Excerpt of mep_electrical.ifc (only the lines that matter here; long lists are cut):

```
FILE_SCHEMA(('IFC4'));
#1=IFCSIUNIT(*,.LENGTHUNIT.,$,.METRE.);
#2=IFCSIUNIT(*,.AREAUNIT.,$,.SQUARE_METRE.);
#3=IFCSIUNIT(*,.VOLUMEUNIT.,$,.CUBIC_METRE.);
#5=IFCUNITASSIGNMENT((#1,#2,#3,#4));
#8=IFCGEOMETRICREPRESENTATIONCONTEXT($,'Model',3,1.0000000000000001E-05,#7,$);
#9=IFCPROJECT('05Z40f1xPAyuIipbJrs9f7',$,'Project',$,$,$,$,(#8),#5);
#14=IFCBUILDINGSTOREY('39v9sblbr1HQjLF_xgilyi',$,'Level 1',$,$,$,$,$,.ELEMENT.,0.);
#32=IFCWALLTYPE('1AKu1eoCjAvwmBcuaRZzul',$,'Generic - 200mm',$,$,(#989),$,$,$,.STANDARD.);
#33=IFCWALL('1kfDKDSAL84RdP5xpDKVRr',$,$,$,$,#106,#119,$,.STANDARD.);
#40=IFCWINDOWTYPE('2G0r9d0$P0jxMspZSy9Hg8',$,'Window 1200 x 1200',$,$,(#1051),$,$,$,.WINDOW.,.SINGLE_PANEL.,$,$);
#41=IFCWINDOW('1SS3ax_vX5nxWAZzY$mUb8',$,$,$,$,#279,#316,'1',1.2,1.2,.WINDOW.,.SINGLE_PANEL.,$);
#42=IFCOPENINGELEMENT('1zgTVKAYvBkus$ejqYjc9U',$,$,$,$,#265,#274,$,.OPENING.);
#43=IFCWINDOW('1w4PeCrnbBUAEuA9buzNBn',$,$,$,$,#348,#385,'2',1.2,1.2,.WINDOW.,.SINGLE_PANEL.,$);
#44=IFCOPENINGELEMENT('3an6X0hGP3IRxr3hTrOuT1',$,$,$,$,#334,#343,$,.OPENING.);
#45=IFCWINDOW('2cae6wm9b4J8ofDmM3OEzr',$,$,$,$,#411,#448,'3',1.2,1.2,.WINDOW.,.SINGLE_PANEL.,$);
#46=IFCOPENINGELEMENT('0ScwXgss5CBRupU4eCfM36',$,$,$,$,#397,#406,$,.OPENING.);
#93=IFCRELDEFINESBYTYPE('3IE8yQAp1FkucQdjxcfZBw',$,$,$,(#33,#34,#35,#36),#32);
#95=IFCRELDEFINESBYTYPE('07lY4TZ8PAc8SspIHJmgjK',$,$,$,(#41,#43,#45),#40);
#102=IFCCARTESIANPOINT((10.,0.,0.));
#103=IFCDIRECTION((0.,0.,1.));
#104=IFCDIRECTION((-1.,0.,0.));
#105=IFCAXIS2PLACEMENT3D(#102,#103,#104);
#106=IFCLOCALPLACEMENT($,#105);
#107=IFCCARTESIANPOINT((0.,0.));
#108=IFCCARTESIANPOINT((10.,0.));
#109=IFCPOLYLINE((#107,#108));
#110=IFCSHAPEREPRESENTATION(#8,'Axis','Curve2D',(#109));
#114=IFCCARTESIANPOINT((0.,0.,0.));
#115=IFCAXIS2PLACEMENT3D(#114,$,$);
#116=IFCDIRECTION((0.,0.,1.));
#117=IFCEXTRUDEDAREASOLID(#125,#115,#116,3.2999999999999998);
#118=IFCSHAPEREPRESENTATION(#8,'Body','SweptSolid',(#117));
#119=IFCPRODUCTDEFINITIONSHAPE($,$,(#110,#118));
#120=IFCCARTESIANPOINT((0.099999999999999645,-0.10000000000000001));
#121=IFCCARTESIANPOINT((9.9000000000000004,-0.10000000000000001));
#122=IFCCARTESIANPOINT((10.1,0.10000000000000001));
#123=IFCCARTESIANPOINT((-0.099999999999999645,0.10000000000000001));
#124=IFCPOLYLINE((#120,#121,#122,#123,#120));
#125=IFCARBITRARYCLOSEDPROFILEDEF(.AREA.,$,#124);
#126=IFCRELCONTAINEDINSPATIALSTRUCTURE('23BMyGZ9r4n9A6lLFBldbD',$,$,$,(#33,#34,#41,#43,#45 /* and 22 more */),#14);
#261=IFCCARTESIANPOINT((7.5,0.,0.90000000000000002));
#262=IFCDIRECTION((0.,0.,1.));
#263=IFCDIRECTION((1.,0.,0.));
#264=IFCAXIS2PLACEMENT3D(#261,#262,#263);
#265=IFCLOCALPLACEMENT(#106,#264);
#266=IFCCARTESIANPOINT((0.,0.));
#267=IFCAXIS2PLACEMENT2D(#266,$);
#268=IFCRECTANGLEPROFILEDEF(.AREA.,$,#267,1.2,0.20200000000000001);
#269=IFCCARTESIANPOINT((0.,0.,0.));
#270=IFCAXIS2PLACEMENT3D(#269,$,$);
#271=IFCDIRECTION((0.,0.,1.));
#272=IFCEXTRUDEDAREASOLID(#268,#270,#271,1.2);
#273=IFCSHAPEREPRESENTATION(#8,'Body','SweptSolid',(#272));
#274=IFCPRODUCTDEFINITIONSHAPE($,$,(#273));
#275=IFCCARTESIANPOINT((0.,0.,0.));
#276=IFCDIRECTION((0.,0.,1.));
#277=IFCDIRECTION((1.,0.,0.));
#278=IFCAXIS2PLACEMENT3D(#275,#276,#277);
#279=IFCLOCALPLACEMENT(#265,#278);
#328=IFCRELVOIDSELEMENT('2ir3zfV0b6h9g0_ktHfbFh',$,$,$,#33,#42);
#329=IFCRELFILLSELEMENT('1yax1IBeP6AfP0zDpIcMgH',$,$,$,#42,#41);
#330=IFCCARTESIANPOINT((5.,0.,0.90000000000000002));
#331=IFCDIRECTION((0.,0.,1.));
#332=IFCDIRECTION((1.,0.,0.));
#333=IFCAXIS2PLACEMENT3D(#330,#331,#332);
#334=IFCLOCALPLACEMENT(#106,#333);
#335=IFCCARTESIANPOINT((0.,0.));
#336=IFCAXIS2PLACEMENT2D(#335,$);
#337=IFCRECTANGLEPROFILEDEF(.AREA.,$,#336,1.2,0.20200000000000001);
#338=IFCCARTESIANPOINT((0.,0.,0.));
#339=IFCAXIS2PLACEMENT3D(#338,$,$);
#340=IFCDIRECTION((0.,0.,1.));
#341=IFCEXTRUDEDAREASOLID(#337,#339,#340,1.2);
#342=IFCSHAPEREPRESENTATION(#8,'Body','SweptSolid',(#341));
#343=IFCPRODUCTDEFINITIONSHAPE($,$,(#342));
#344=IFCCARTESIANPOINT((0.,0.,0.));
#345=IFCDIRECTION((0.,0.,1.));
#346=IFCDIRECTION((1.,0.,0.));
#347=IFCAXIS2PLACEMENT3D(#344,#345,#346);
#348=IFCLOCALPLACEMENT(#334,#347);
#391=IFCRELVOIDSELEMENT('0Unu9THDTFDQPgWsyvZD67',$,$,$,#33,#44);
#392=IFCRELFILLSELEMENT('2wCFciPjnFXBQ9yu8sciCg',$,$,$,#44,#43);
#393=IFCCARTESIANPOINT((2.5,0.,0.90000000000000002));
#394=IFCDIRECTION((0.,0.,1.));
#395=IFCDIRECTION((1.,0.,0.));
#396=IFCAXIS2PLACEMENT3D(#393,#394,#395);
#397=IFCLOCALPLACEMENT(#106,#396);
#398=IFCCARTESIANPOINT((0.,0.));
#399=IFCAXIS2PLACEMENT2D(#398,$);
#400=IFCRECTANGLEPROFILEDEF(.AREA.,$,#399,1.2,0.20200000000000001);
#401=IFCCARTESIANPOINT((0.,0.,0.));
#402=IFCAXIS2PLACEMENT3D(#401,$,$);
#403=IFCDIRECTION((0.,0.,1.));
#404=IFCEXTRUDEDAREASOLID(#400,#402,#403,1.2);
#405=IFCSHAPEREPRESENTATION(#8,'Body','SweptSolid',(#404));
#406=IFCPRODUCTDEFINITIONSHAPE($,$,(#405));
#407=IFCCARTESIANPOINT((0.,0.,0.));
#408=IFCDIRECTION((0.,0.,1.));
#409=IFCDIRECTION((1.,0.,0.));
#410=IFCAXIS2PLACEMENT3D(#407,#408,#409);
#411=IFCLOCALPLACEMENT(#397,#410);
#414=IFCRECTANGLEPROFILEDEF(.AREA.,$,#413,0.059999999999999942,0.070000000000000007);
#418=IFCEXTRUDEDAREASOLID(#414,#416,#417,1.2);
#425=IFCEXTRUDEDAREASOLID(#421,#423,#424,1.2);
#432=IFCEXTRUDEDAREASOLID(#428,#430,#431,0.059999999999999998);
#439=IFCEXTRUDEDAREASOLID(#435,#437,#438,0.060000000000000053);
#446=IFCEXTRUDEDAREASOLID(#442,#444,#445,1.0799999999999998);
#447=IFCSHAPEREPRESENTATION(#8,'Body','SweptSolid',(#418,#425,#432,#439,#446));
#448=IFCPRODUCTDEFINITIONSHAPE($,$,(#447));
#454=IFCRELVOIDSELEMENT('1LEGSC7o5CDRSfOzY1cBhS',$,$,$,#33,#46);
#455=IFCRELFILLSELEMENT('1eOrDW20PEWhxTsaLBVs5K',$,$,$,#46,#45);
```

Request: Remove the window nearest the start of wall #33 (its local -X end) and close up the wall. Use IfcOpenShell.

```python
import ifcopenshell
import ifcopenshell.api.feature
import ifcopenshell.api.root
import ifcopenshell.geom
import ifcopenshell.util.shape

model = ifcopenshell.open("mep_electrical.ifc")
settings = ifcopenshell.geom.settings()


def volume(element):
    """Net volume in cubic metres, openings subtracted."""
    shape = ifcopenshell.geom.create_shape(settings, element)
    return ifcopenshell.util.shape.get_volume(shape.geometry)


window = model.by_id(45)
opening = window.FillsVoids[0].RelatingOpeningElement
wall = opening.VoidsElements[0].RelatingBuildingElement
before = volume(wall)

ifcopenshell.api.root.remove_product(model, product=window)
ifcopenshell.api.feature.remove_feature(model, feature=opening)

after = volume(wall)

print(f"wall volume {before:.3f} -> {after:.3f} m3")

model.write("mep_electrical_updated.ifc")
```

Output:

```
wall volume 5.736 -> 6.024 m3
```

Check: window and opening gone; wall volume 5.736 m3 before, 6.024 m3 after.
